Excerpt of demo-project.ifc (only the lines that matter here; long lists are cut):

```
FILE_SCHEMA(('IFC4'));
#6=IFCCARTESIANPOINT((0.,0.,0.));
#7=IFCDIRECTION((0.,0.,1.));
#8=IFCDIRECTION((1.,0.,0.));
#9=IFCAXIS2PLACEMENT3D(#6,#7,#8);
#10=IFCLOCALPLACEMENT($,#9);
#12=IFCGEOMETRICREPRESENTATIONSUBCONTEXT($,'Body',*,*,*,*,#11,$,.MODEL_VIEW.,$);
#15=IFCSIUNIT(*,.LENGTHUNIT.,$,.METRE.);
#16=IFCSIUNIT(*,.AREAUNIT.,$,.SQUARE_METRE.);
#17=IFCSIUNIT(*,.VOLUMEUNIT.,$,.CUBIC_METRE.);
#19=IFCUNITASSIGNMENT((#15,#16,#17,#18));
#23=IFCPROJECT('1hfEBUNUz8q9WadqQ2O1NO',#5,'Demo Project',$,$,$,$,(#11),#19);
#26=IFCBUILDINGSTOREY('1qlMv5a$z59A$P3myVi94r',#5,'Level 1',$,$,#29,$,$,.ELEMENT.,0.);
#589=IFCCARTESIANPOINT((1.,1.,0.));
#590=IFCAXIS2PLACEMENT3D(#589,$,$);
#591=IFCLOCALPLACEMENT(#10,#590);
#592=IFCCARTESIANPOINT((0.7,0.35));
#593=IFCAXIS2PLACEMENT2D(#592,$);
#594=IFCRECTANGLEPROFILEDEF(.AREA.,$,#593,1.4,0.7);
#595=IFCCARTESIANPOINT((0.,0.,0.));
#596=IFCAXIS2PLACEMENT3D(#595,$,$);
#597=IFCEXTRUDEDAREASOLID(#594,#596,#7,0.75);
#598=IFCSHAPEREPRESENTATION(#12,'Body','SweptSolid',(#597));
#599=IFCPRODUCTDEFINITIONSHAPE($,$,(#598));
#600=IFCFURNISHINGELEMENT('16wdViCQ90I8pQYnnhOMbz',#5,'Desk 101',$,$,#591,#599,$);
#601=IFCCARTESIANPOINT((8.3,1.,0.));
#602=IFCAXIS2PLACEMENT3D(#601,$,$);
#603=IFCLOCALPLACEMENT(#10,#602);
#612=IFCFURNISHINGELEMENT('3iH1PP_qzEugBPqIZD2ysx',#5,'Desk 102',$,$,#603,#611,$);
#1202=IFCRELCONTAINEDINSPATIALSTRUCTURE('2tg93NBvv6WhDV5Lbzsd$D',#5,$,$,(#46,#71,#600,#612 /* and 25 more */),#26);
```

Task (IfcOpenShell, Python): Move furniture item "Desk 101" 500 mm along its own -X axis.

```python
import ifcopenshell
import ifcopenshell.api.geometry
import ifcopenshell.util.placement

model = ifcopenshell.open("demo-project.ifc")

item = model.by_guid("16wdViCQ90I8pQYnnhOMbz")
matrix = ifcopenshell.util.placement.get_local_placement(item.ObjectPlacement)
matrix[:3, 3] -= matrix[:3, 0] * 0.5
ifcopenshell.api.geometry.edit_object_placement(model, product=item, matrix=matrix, is_si=False)

print(ifcopenshell.util.placement.get_local_placement(item.ObjectPlacement).round(3) + 0.0)

model.write("demo-project_v2.ifc")
```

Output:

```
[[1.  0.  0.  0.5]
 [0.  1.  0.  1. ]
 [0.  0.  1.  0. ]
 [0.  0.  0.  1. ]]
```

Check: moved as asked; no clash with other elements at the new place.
